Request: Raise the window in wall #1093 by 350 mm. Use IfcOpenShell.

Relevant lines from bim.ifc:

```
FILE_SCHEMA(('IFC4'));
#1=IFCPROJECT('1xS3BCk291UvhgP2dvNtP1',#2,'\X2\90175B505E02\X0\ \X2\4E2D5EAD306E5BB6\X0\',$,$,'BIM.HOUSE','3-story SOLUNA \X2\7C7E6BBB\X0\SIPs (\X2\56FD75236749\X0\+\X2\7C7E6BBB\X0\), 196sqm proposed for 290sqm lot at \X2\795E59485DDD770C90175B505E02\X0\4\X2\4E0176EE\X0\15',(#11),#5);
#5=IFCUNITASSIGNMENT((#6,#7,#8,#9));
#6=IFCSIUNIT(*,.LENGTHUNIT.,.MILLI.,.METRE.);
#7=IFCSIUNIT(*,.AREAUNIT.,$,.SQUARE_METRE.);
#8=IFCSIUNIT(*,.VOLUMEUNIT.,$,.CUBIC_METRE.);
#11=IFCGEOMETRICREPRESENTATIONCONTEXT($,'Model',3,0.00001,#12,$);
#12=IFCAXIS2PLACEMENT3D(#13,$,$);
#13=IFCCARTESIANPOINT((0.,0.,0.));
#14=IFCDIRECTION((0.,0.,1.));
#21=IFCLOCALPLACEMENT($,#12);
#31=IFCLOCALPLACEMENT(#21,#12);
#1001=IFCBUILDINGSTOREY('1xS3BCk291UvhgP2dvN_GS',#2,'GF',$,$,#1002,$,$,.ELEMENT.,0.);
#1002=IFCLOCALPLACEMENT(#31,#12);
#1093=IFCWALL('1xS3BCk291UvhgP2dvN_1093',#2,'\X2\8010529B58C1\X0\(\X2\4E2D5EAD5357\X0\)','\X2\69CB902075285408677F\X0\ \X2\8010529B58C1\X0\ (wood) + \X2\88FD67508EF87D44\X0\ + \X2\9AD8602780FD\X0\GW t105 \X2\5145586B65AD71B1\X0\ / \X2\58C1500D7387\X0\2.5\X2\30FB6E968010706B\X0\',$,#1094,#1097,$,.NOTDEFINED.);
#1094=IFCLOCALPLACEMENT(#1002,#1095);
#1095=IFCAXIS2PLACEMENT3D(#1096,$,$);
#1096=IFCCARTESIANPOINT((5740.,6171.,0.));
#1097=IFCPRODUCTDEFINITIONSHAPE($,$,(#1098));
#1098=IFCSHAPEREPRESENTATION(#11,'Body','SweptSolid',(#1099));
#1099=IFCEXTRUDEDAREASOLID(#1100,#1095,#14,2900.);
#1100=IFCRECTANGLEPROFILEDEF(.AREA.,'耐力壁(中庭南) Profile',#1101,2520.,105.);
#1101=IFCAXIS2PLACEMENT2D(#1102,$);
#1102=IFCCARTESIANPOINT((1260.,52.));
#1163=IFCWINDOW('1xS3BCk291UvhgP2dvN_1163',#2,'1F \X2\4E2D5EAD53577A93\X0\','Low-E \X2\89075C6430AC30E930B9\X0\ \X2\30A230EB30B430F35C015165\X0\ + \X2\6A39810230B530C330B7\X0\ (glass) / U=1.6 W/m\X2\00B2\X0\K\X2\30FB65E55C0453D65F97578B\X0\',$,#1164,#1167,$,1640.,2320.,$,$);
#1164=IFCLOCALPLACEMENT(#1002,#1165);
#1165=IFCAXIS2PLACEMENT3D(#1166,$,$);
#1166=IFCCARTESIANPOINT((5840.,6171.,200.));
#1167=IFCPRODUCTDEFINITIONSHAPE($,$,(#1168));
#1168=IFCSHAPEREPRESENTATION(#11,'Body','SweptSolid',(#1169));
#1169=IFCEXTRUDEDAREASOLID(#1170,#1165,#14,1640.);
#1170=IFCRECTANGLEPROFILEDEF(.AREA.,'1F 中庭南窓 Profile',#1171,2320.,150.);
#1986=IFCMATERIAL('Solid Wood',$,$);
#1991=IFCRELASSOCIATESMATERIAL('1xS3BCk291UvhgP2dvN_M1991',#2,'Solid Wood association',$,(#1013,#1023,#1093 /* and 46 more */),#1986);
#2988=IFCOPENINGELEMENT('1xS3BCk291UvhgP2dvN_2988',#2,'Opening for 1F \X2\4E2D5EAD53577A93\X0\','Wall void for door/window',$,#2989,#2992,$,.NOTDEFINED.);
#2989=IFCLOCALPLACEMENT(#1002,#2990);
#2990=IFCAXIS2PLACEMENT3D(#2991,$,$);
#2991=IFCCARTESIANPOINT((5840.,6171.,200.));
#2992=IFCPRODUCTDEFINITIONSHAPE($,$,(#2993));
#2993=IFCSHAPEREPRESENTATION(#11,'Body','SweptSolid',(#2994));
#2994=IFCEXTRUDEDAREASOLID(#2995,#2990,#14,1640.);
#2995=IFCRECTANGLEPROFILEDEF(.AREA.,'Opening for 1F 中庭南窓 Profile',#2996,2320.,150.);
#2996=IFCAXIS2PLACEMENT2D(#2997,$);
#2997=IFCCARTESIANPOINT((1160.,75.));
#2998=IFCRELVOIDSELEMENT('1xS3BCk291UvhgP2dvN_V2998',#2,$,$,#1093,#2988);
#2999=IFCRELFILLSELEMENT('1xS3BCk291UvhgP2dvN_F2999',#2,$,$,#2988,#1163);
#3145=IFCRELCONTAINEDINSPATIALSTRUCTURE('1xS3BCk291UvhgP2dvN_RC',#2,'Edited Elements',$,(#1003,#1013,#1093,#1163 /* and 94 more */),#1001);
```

```python
import numpy as np
import ifcopenshell
import ifcopenshell.api.geometry
import ifcopenshell.util.placement
import ifcopenshell.util.unit

model = ifcopenshell.open("bim.ifc")
unit_scale = ifcopenshell.util.unit.calculate_unit_scale(model)

window = model.by_guid("1xS3BCk291UvhgP2dvN_1163")
opening = window.FillsVoids[0].RelatingOpeningElement
dz = 0.35 / unit_scale

shift = np.array([0.0, 0.0, dz])
# The window is not placed relative to its opening, so move both.
for product in (opening, window):
    matrix = ifcopenshell.util.placement.get_local_placement(product.ObjectPlacement)
    matrix[:3, 3] += shift
    ifcopenshell.api.geometry.edit_object_placement(model, product=product, matrix=matrix, is_si=False)

print(f"moved by {dz * unit_scale:+.3f} m")

model.write("bim_v2.ifc")
```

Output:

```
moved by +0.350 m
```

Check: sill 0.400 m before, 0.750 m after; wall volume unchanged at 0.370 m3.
